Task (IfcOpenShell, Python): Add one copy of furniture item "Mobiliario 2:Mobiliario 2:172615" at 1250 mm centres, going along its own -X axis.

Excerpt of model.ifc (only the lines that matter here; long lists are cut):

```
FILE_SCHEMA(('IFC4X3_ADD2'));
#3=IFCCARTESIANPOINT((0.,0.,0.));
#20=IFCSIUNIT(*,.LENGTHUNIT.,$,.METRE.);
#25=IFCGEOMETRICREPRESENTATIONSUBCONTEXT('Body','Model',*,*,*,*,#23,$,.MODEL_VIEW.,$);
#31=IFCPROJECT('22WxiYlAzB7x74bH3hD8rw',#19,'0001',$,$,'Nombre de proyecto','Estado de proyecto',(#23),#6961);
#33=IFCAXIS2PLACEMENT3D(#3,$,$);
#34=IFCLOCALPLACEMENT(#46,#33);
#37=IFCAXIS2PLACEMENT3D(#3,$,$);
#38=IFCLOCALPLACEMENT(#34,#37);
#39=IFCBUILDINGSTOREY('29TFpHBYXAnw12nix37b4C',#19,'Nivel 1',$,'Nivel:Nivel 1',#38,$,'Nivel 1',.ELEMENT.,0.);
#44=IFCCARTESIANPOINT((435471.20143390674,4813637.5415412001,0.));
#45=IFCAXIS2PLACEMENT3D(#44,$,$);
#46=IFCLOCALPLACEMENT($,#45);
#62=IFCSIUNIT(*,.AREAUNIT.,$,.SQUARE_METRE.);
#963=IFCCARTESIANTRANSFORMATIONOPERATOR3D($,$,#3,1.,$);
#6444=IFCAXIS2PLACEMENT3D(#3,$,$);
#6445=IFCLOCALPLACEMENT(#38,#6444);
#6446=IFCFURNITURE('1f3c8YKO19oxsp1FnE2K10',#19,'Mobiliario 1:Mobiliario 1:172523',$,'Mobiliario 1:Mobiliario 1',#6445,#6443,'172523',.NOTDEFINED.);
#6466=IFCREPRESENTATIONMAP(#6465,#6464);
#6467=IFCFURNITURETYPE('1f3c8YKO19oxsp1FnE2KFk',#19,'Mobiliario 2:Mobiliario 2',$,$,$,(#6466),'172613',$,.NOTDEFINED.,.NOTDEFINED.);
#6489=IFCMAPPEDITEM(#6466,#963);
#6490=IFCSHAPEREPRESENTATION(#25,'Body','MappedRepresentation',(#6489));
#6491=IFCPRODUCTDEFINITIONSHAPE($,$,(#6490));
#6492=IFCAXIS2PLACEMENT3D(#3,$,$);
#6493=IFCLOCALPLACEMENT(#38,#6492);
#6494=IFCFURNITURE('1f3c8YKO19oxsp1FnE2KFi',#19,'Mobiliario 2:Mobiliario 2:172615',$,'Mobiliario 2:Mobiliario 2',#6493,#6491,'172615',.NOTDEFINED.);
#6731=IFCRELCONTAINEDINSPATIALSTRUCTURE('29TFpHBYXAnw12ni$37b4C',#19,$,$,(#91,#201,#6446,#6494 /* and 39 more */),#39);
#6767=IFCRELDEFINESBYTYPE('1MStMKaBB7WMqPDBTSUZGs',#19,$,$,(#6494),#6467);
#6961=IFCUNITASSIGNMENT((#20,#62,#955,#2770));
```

```python
import ifcopenshell
import ifcopenshell.api.geometry
import ifcopenshell.api.root
import ifcopenshell.util.element
import ifcopenshell.util.placement
import ifcopenshell.util.unit

model = ifcopenshell.open("model.ifc")
unit_scale = ifcopenshell.util.unit.calculate_unit_scale(model)


def reuse_history(source, copy):
    """copy_class also copies each property set's owner history, people and application; keep the originals."""
    for rel in copy.IsDefinedBy:
        if rel.is_a("IfcRelDefinesByProperties") and (history := rel.RelatingPropertyDefinition.OwnerHistory):
            rel.RelatingPropertyDefinition.OwnerHistory = source.OwnerHistory
            ifcopenshell.util.element.remove_deep2(model, history)


source = model.by_guid("1f3c8YKO19oxsp1FnE2KFi")
base = ifcopenshell.util.placement.get_local_placement(source.ObjectPlacement)
step = -base[:3, 0] * 1.25 / unit_scale

for i in range(1, 2):
    copy = ifcopenshell.api.root.copy_class(model, product=source)
    copy.Representation = ifcopenshell.util.element.copy_deep(
        model, source.Representation, exclude=["IfcGeometricRepresentationContext", "IfcRepresentationMap"]
    )
    copy.Name = "Mobiliario 2:Mobiliario 2"
    copy.Tag = None
    reuse_history(source, copy)
    matrix = base.copy()
    matrix[:3, 3] += i * step
    print("added at", matrix[:3, 3].round(3) + 0.0)
    ifcopenshell.api.geometry.edit_object_placement(model, product=copy, matrix=matrix, is_si=False)

model.write("model_edited.ifc")
```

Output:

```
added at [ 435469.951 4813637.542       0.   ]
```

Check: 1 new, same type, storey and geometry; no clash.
